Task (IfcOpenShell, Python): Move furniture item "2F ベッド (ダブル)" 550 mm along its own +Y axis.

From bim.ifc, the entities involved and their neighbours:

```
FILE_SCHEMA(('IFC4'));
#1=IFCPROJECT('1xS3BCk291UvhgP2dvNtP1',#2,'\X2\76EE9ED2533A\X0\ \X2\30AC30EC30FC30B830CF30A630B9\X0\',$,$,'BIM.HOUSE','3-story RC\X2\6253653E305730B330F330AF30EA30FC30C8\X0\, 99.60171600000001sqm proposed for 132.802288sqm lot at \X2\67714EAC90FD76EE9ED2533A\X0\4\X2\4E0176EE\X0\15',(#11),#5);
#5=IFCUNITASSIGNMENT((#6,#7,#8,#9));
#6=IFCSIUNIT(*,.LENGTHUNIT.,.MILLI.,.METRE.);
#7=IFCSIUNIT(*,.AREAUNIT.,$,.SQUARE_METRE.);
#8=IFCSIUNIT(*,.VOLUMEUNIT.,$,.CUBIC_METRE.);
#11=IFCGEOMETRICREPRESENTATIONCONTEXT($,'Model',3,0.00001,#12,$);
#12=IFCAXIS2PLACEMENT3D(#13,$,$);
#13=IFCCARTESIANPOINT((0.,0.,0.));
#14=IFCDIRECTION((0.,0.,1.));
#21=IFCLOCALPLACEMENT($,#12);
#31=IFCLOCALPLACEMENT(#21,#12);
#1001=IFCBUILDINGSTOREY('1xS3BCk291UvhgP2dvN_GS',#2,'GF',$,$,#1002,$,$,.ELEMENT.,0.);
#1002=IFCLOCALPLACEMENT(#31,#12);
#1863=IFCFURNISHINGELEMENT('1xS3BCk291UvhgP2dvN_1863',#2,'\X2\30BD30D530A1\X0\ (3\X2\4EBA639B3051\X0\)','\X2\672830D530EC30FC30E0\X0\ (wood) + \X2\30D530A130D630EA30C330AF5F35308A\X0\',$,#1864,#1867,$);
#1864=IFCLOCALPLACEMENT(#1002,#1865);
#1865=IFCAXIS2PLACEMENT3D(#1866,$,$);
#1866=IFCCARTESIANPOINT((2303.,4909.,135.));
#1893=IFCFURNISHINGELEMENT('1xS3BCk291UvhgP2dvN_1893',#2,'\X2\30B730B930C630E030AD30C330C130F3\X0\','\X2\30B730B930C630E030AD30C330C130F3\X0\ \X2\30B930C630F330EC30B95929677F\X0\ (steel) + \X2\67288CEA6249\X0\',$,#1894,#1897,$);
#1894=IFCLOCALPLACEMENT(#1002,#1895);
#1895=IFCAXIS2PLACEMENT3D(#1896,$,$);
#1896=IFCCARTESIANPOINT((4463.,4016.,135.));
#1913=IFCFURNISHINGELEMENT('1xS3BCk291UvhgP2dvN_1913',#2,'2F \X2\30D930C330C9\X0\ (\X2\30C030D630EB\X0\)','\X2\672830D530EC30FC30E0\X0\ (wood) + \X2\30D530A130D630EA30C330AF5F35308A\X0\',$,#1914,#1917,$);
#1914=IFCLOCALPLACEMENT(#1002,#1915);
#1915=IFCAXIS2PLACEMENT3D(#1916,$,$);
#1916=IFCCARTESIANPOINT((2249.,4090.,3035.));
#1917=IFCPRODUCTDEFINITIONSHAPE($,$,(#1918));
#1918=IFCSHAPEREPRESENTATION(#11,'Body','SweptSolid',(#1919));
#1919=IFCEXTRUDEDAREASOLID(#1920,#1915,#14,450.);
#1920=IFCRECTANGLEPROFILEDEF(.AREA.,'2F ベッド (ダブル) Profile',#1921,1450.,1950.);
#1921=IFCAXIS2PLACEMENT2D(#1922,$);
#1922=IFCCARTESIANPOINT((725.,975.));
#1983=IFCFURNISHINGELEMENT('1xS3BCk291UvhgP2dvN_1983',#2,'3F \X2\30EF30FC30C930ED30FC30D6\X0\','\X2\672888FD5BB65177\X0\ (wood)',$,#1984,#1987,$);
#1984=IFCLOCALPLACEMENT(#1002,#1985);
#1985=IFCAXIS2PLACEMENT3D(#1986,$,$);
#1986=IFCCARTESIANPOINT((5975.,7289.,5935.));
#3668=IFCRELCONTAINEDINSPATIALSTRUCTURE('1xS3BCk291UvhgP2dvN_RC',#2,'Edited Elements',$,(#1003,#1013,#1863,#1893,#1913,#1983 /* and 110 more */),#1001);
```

```python
import ifcopenshell
import ifcopenshell.api.geometry
import ifcopenshell.util.placement
import ifcopenshell.util.unit

model = ifcopenshell.open("bim.ifc")
unit_scale = ifcopenshell.util.unit.calculate_unit_scale(model)

item = model.by_guid("1xS3BCk291UvhgP2dvN_1913")
matrix = ifcopenshell.util.placement.get_local_placement(item.ObjectPlacement)
matrix[:3, 3] += matrix[:3, 1] * 0.55 / unit_scale
ifcopenshell.api.geometry.edit_object_placement(model, product=item, matrix=matrix, is_si=False)

print(ifcopenshell.util.placement.get_local_placement(item.ObjectPlacement).round(3) + 0.0)

model.write("bim_v2.ifc")
```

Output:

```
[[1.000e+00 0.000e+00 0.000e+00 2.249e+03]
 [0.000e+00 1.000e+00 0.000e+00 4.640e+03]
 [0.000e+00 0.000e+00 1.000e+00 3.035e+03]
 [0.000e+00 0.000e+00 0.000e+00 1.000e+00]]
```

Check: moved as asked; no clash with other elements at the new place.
